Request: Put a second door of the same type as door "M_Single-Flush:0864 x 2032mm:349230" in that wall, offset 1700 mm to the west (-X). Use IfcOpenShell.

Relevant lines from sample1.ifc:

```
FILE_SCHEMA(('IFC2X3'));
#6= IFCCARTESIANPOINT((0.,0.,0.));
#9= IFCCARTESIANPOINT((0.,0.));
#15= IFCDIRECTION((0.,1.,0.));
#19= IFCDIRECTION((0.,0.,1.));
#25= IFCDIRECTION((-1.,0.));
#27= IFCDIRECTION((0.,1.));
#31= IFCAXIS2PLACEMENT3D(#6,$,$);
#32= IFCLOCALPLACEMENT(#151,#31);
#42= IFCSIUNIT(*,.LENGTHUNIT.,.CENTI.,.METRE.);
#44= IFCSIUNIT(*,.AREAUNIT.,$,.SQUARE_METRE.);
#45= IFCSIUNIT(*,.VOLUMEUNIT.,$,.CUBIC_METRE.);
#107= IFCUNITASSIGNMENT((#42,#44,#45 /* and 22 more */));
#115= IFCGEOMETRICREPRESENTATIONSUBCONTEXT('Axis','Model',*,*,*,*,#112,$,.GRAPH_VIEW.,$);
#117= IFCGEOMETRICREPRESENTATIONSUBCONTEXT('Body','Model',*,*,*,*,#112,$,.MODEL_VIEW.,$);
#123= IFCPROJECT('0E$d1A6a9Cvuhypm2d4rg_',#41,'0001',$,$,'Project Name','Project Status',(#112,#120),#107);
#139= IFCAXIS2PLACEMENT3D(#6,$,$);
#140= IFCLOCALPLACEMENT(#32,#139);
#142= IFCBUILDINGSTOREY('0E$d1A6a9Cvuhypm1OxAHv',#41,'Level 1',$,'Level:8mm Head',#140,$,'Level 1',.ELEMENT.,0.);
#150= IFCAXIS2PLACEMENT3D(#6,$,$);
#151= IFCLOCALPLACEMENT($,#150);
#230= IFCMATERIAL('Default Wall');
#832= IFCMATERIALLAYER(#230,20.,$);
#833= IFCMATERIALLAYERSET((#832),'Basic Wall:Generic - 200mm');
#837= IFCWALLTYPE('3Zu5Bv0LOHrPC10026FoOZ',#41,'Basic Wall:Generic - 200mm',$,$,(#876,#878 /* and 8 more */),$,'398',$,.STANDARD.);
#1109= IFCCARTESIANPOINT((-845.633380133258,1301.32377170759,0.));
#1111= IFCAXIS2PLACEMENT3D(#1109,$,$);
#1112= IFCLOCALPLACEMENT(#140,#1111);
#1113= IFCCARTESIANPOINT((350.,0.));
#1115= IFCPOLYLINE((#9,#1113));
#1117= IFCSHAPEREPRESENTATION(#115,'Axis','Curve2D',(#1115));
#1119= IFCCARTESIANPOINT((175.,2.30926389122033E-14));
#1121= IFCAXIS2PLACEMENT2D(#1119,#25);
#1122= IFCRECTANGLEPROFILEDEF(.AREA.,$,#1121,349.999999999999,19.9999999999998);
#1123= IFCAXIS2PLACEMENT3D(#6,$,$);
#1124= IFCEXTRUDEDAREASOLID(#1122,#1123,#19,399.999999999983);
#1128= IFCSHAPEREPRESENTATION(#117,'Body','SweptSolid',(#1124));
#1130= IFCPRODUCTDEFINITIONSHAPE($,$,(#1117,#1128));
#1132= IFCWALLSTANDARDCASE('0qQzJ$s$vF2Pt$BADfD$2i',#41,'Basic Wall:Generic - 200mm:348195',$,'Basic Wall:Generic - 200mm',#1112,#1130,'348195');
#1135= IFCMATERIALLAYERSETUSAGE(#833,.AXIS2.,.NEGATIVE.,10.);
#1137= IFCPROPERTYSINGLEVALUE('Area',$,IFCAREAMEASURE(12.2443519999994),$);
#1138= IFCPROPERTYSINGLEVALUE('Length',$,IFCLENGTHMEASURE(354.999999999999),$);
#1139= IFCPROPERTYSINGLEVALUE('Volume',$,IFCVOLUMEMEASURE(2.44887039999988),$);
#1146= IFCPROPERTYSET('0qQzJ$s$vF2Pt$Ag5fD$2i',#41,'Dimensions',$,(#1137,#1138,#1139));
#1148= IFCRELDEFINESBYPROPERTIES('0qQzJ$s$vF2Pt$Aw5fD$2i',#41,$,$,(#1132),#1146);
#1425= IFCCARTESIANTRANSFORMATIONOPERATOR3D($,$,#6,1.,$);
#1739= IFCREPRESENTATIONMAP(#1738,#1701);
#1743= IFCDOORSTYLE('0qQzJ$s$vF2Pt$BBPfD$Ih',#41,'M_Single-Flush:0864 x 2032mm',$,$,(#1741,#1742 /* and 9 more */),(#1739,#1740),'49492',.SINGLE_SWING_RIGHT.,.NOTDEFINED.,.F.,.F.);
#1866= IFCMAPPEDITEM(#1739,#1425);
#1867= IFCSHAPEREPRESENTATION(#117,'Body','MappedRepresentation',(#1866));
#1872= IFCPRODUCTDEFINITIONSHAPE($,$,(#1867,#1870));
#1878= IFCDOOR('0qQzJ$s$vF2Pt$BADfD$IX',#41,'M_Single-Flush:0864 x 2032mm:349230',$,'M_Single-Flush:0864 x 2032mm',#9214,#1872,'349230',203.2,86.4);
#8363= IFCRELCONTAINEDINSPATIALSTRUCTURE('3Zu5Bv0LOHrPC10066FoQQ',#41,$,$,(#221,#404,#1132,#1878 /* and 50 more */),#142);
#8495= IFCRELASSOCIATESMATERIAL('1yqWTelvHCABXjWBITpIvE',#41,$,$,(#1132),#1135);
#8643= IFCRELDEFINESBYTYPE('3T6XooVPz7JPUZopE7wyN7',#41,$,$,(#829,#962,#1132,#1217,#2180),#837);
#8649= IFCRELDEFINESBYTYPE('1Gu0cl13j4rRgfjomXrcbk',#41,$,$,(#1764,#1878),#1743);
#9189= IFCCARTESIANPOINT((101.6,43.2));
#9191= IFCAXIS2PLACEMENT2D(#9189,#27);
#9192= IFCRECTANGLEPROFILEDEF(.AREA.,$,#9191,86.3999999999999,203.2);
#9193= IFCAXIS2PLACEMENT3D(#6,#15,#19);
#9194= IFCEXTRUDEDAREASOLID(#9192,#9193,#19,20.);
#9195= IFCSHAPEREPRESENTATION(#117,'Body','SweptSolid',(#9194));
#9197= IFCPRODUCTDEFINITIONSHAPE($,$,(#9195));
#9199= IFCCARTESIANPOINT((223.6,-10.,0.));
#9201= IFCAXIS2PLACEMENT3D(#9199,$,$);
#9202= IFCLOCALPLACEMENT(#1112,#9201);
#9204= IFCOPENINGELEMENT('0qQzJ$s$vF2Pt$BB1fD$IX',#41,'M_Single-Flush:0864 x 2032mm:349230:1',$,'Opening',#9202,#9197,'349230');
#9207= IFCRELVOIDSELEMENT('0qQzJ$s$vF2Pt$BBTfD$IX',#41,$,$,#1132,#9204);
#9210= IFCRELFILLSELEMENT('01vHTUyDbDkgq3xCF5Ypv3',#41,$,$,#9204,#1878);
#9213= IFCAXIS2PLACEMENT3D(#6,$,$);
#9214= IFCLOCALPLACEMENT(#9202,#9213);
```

```python
import ifcopenshell
import ifcopenshell.api.feature
import ifcopenshell.api.geometry
import ifcopenshell.api.pset
import ifcopenshell.api.root
import ifcopenshell.geom
import ifcopenshell.util.element
import ifcopenshell.util.placement
import ifcopenshell.util.shape
import ifcopenshell.util.unit

model = ifcopenshell.open("sample1.ifc")
unit_scale = ifcopenshell.util.unit.calculate_unit_scale(model)
area_scale = ifcopenshell.util.unit.calculate_unit_scale(model, "AREAUNIT")
volume_scale = ifcopenshell.util.unit.calculate_unit_scale(model, "VOLUMEUNIT")
settings = ifcopenshell.geom.settings()


def volume(element):
    """Net volume in cubic metres, openings subtracted."""
    shape = ifcopenshell.geom.create_shape(settings, element)
    return ifcopenshell.util.shape.get_volume(shape.geometry)


def reuse_history(source, copy):
    """copy_class also copies each property set's owner history, people and application; keep the originals."""
    for rel in copy.IsDefinedBy:
        if rel.is_a("IfcRelDefinesByProperties") and (history := rel.RelatingPropertyDefinition.OwnerHistory):
            rel.RelatingPropertyDefinition.OwnerHistory = source.OwnerHistory
            ifcopenshell.util.element.remove_deep2(model, history)


door = model.by_guid("0qQzJ$s$vF2Pt$BADfD$IX")
opening = door.FillsVoids[0].RelatingOpeningElement
wall = opening.VoidsElements[0].RelatingBuildingElement
before = volume(wall)
shift = ifcopenshell.util.placement.get_local_placement(wall.ObjectPlacement)[:3, 0] * -1.7 / unit_scale

# copy_class copies the void relationship, type, container and properties, but no geometry.
new_opening = ifcopenshell.api.root.copy_class(model, product=opening)
new_opening.Representation = ifcopenshell.util.element.copy_deep(
    model, opening.Representation, exclude=["IfcGeometricRepresentationContext", "IfcRepresentationMap"]
)
new_opening.Name = "M_Single-Flush:0864 x 2032mm"
new_opening.Tag = None
new_door = ifcopenshell.api.root.copy_class(model, product=door)
new_door.Representation = ifcopenshell.util.element.copy_deep(
    model, door.Representation, exclude=["IfcGeometricRepresentationContext", "IfcRepresentationMap"]
)
new_door.Name = "M_Single-Flush:0864 x 2032mm"
new_door.Tag = None
reuse_history(door, new_door)
fills = ifcopenshell.api.feature.add_filling(model, opening=new_opening, element=new_door)
fills.OwnerHistory = new_door.OwnerHistory  # required in IFC2X3

for old, new in ((opening, new_opening), (door, new_door)):
    matrix = ifcopenshell.util.placement.get_local_placement(old.ObjectPlacement)
    matrix[:3, 3] += shift
    ifcopenshell.api.geometry.edit_object_placement(model, product=new, matrix=matrix, is_si=False)

after = volume(wall)
thickness = 0.2  # wall thickness in metres

# Update the wall's stored quantities.
pset = model.by_id(ifcopenshell.util.element.get_pset(wall, "Dimensions", should_inherit=False)["id"])
ifcopenshell.api.pset.edit_pset(model, pset=pset, properties={
    "Area": model.create_entity("IfcAreaMeasure", after / thickness / area_scale),
    "Volume": model.create_entity("IfcVolumeMeasure", after / volume_scale),
})

print(f"wall volume {before:.3f} -> {after:.3f} m3")

model.write("sample1_rev.ifc")
```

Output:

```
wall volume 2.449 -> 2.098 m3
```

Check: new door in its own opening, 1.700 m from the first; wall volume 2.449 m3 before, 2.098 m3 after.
